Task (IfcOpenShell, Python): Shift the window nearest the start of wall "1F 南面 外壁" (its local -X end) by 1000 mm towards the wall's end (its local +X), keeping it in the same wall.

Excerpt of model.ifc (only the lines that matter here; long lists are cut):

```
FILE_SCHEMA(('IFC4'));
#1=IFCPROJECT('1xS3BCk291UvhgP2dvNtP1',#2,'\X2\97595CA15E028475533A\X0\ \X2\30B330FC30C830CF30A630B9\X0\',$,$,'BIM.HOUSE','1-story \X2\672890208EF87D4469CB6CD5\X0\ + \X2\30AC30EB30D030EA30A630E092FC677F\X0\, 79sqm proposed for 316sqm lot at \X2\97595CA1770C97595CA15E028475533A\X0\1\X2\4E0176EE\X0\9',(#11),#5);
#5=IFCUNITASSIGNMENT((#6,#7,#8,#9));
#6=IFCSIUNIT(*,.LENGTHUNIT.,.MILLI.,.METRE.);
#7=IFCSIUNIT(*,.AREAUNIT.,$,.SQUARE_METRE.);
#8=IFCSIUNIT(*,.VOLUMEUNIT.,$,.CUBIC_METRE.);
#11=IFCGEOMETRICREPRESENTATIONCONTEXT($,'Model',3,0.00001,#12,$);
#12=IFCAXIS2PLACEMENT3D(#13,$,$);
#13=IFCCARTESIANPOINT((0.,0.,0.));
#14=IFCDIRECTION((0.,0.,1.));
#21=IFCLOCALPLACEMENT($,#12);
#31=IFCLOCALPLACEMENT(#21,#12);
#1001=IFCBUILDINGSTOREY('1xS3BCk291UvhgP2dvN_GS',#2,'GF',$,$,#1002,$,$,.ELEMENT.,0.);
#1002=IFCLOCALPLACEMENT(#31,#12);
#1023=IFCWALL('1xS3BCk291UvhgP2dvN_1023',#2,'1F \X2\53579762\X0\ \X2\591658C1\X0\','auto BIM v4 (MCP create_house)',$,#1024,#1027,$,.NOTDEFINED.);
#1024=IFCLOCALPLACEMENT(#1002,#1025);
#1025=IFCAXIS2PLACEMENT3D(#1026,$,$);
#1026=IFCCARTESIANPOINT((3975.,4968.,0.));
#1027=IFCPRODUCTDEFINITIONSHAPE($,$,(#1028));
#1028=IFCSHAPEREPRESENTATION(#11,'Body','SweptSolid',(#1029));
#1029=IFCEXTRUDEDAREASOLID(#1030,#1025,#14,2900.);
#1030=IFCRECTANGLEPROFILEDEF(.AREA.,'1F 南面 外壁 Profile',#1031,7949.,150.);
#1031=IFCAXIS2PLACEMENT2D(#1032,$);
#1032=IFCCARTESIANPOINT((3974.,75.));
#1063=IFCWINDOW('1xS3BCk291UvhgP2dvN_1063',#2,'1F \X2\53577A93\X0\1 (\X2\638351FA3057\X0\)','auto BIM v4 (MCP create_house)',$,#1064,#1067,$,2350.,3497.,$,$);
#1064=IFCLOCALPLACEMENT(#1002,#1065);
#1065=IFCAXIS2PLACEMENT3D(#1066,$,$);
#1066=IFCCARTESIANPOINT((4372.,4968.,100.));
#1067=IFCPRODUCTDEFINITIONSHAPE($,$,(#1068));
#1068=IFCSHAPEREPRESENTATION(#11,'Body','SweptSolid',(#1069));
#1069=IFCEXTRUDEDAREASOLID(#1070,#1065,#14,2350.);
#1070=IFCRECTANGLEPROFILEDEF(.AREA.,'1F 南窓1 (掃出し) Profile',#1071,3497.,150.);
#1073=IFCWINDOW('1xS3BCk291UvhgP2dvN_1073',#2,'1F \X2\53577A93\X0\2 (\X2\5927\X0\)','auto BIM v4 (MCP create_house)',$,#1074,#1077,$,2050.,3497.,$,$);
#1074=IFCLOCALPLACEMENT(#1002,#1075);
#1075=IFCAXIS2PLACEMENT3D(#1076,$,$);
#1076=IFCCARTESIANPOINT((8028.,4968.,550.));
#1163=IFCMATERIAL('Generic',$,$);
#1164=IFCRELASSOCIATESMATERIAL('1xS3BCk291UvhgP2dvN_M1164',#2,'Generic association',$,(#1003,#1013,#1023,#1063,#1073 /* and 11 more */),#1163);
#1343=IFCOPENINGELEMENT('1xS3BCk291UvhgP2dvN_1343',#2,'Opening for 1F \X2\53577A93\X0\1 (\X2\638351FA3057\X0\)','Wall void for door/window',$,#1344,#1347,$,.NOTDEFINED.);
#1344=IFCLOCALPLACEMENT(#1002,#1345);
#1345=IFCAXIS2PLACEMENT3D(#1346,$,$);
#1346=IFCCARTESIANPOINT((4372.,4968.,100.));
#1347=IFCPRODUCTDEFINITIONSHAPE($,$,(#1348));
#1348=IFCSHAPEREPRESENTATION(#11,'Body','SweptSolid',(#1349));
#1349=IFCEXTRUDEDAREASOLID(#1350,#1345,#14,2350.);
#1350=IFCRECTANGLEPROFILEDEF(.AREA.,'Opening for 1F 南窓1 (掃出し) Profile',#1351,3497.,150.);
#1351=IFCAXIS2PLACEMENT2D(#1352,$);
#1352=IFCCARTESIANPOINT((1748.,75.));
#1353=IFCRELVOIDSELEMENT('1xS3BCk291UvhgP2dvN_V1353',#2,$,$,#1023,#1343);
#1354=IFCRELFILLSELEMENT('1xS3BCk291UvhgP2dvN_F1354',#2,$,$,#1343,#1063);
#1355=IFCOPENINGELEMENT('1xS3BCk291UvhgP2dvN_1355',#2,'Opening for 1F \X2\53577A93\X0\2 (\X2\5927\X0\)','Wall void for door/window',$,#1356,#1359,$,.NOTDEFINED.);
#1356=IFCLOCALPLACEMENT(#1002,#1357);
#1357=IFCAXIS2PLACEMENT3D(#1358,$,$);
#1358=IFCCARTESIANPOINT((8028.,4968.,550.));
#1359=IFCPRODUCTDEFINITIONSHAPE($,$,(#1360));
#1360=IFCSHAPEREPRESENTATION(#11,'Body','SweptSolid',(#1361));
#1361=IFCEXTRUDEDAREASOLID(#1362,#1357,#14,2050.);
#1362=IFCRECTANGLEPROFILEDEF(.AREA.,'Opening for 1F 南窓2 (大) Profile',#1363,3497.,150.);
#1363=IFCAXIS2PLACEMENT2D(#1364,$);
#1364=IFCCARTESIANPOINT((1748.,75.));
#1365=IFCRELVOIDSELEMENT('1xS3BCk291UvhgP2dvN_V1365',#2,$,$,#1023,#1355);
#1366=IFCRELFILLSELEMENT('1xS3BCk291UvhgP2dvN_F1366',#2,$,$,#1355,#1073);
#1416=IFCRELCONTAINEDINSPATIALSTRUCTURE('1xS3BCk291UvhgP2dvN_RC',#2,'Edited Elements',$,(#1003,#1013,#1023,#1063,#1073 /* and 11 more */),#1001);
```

```python
import ifcopenshell
import ifcopenshell.api.geometry
import ifcopenshell.util.placement

model = ifcopenshell.open("model.ifc")

window = model.by_id(1063)
opening = window.FillsVoids[0].RelatingOpeningElement
wall = opening.VoidsElements[0].RelatingBuildingElement

wall_matrix = ifcopenshell.util.placement.get_local_placement(wall.ObjectPlacement)
shift = wall_matrix[:3, 0] * 1000.0
before = ifcopenshell.util.placement.get_local_placement(window.ObjectPlacement)[:3, 3].copy()

# The window is not placed relative to its opening, so move both.
for product in (opening, window):
    matrix = ifcopenshell.util.placement.get_local_placement(product.ObjectPlacement)
    matrix[:3, 3] += shift
    ifcopenshell.api.geometry.edit_object_placement(model, product=product, matrix=matrix, is_si=False)

after = ifcopenshell.util.placement.get_local_placement(window.ObjectPlacement)[:3, 3]
print("window moved by", (after - before).round(3) + 0.0)

model.write("model-out.ifc")
```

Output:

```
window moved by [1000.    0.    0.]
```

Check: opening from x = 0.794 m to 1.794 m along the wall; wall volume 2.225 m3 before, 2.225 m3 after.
